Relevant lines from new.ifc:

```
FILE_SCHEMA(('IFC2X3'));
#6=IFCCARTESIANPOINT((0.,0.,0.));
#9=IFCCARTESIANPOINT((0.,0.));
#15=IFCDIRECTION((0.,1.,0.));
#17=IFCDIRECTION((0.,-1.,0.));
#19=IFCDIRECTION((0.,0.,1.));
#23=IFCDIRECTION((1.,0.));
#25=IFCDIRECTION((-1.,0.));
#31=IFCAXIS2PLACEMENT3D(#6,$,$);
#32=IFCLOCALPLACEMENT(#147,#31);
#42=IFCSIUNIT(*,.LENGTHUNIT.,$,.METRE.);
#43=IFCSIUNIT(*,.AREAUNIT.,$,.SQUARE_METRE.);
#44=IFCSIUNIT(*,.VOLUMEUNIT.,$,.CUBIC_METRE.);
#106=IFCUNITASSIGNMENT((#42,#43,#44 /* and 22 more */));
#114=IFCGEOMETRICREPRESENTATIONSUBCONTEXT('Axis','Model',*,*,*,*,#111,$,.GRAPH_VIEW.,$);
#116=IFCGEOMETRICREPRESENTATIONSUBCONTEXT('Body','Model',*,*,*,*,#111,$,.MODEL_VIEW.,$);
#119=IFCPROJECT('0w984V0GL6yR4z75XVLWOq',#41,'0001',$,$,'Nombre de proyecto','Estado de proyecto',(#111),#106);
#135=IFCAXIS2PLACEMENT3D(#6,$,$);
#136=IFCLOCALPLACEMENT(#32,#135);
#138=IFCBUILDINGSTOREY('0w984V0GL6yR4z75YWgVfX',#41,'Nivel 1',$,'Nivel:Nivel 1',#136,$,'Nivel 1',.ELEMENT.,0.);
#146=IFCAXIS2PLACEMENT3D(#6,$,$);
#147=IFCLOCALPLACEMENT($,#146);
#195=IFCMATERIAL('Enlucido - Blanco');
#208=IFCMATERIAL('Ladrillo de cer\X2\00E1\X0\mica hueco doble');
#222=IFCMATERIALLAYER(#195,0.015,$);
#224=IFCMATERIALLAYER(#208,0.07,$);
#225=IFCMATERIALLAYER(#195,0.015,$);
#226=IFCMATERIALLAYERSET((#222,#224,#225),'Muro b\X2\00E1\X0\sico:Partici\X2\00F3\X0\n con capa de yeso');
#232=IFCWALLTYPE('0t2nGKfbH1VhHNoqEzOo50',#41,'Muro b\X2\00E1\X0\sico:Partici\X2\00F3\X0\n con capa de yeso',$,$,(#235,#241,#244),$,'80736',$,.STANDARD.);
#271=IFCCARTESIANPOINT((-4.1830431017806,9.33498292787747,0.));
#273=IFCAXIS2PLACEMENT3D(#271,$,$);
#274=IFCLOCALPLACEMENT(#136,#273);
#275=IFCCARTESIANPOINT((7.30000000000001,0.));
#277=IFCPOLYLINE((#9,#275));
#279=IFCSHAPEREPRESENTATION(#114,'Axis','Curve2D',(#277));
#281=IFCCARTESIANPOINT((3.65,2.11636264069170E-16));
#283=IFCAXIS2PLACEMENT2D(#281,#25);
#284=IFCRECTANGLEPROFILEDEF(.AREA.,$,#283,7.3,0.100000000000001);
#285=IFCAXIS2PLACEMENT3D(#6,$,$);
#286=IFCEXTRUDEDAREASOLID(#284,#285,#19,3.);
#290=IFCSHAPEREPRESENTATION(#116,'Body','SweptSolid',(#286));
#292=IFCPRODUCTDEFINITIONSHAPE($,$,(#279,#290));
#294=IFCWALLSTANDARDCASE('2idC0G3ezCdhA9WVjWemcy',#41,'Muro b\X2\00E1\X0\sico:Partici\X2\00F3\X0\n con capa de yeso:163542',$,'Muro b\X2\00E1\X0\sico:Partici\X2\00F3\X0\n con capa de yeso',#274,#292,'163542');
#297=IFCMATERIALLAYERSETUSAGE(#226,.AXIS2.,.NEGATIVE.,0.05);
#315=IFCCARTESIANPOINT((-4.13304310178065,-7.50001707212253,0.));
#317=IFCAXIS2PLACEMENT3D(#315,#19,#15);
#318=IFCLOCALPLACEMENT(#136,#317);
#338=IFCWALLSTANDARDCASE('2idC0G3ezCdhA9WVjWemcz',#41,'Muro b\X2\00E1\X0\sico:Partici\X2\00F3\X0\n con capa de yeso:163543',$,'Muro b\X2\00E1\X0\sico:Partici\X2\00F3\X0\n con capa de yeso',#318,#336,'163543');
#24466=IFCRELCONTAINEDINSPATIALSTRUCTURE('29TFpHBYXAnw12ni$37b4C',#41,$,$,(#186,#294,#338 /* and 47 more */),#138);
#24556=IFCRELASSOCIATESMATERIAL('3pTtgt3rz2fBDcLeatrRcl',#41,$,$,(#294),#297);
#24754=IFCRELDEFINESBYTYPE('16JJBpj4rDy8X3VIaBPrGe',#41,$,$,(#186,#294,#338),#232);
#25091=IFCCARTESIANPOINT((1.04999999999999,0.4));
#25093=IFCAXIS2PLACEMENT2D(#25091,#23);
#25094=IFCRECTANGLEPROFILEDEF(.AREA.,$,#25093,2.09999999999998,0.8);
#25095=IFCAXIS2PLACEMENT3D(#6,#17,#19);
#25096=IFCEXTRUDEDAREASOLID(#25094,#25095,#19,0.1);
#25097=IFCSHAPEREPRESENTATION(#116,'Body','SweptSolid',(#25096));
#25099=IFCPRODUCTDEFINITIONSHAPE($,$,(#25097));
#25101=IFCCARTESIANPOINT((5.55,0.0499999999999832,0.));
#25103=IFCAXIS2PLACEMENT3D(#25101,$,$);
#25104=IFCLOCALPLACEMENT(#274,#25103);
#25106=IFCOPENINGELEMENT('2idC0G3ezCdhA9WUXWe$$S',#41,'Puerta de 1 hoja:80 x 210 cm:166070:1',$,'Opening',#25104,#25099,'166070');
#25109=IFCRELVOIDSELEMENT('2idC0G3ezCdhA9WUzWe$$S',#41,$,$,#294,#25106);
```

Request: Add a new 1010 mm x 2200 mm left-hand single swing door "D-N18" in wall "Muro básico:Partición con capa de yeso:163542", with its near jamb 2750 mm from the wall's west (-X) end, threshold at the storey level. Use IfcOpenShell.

```python
import numpy as np
import ifcopenshell
import ifcopenshell.api.feature
import ifcopenshell.api.geometry
import ifcopenshell.api.root
import ifcopenshell.api.spatial
import ifcopenshell.api.type
import ifcopenshell.geom
import ifcopenshell.util.element
import ifcopenshell.util.placement
import ifcopenshell.util.representation
import ifcopenshell.util.shape
import ifcopenshell.util.unit

model = ifcopenshell.open("new.ifc")
unit_scale = ifcopenshell.util.unit.calculate_unit_scale(model)
settings = ifcopenshell.geom.settings()


def volume(element):
    """Net volume in cubic metres, openings subtracted."""
    shape = ifcopenshell.geom.create_shape(settings, element)
    return ifcopenshell.util.shape.get_volume(shape.geometry)


wall = model.by_guid("2idC0G3ezCdhA9WVjWemcy")
storey = ifcopenshell.util.element.get_container(wall, ifc_class="IfcBuildingStorey")
context = ifcopenshell.util.representation.get_context(model, "Model", "Body", "MODEL_VIEW")
before = volume(wall)

width, height, from_end, sill = 1.01, 2.2, 2.75, 0.0  # metres

# The wall runs along its own X axis, and the end named is its -X end.
wall_shape = ifcopenshell.geom.create_shape(settings, wall)
x, y, z = ifcopenshell.util.shape.get_vertices(wall_shape.geometry).T
start = x.min() + from_end
face, thickness = float(y.min()), float(y.max() - y.min())
wall_matrix = ifcopenshell.util.placement.get_local_placement(wall.ObjectPlacement)
level = ifcopenshell.util.placement.get_local_placement(storey.ObjectPlacement)[2, 3]


def in_wall(x, y):
    """Placement at x, y metres in the wall's axes, at sill height."""
    matrix = wall_matrix.copy()
    matrix[:, 3] = wall_matrix @ np.array([x / unit_scale, y / unit_scale, 0.0, 1.0])
    matrix[2, 3] = level + sill / unit_scale
    return matrix


# Opening: a box that overshoots both wall faces by 50 mm.
opening = ifcopenshell.api.root.create_entity(model, ifc_class="IfcOpeningElement")
box = ifcopenshell.api.geometry.add_wall_representation(
    model, context=context, length=width, height=height, thickness=thickness + 0.1
)
ifcopenshell.api.geometry.assign_representation(model, product=opening, representation=box)
ifcopenshell.api.geometry.edit_object_placement(model, product=opening, matrix=in_wall(start, face - 0.05), is_si=False)
ifcopenshell.api.feature.add_feature(model, feature=opening, element=wall)

door = ifcopenshell.api.root.create_entity(model, ifc_class="IfcDoor", name="D-N18")
door.OverallWidth, door.OverallHeight = width / unit_scale, height / unit_scale
body = ifcopenshell.api.geometry.add_door_representation(
    model,
    context=context,
    overall_width=door.OverallWidth,
    overall_height=door.OverallHeight,
    operation_type="SINGLE_SWING_LEFT",
    lining_properties={"LiningDepth": thickness / unit_scale, "ThresholdDepth": thickness / unit_scale},
)
ifcopenshell.api.geometry.assign_representation(model, product=door, representation=body)
ifcopenshell.api.spatial.assign_container(model, products=[door], relating_structure=storey)
fills = ifcopenshell.api.feature.add_filling(model, opening=opening, element=door)
fills.OwnerHistory = door.OwnerHistory  # required in IFC2X3

# IFC2X3 keeps the operation on the door style.
style = ifcopenshell.api.root.create_entity(model, ifc_class="IfcDoorStyle", name="D-N18")
style.OperationType, style.ConstructionType = "SINGLE_SWING_LEFT", "NOTDEFINED"
style.ParameterTakesPrecedence = style.Sizeable = False
ifcopenshell.api.type.assign_type(model, related_objects=[door], relating_type=style)

# The lining spans the wall, so the door starts at the wall face.
ifcopenshell.api.geometry.edit_object_placement(model, product=door, matrix=in_wall(start, face), is_si=False)

after = volume(wall)

print(f"wall volume {before:.3f} -> {after:.3f} m3")

model.write("new_updated.ifc")
```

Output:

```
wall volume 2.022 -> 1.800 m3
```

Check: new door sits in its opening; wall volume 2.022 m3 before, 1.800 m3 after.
